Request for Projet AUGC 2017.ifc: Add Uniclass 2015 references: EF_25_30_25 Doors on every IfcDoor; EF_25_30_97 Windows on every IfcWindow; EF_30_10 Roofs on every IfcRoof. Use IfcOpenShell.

First a look at what the model holds.

```python
import ifcopenshell

model = ifcopenshell.open("Projet AUGC 2017.ifc")
print(model.schema)
print("classifications:", [c.Name for c in model.by_type("IfcClassification")])
for ifc_class in ("IfcDoor", "IfcRoof", "IfcStair", "IfcWall", "IfcWindow"):
    print(ifc_class, len(model.by_type(ifc_class)))
```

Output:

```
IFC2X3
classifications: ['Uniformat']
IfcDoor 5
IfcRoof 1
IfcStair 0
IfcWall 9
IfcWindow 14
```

```python
import ifcopenshell
import ifcopenshell.api.classification

model = ifcopenshell.open("Projet AUGC 2017.ifc")

# IFC2X3 requires Source and Edition and has no link from the project to the system.
system = model.create_entity("IfcClassification", Source="NBS", Edition="2015", Name="Uniclass 2015")

codes = {
    "IfcDoor": ("EF_25_30_25", "Doors"),
    "IfcWindow": ("EF_25_30_97", "Windows"),
    "IfcRoof": ("EF_30_10", "Roofs"),
}
for ifc_class, (code, name) in codes.items():
    products = model.by_type(ifc_class)
    ifcopenshell.api.classification.add_reference(
        model, products=products, classification=system, identification=code, name=name
    )
    print(code, len(products))

model.write("Projet AUGC 2017_edited.ifc")
```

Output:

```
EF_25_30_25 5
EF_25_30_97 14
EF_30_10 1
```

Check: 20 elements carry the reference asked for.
